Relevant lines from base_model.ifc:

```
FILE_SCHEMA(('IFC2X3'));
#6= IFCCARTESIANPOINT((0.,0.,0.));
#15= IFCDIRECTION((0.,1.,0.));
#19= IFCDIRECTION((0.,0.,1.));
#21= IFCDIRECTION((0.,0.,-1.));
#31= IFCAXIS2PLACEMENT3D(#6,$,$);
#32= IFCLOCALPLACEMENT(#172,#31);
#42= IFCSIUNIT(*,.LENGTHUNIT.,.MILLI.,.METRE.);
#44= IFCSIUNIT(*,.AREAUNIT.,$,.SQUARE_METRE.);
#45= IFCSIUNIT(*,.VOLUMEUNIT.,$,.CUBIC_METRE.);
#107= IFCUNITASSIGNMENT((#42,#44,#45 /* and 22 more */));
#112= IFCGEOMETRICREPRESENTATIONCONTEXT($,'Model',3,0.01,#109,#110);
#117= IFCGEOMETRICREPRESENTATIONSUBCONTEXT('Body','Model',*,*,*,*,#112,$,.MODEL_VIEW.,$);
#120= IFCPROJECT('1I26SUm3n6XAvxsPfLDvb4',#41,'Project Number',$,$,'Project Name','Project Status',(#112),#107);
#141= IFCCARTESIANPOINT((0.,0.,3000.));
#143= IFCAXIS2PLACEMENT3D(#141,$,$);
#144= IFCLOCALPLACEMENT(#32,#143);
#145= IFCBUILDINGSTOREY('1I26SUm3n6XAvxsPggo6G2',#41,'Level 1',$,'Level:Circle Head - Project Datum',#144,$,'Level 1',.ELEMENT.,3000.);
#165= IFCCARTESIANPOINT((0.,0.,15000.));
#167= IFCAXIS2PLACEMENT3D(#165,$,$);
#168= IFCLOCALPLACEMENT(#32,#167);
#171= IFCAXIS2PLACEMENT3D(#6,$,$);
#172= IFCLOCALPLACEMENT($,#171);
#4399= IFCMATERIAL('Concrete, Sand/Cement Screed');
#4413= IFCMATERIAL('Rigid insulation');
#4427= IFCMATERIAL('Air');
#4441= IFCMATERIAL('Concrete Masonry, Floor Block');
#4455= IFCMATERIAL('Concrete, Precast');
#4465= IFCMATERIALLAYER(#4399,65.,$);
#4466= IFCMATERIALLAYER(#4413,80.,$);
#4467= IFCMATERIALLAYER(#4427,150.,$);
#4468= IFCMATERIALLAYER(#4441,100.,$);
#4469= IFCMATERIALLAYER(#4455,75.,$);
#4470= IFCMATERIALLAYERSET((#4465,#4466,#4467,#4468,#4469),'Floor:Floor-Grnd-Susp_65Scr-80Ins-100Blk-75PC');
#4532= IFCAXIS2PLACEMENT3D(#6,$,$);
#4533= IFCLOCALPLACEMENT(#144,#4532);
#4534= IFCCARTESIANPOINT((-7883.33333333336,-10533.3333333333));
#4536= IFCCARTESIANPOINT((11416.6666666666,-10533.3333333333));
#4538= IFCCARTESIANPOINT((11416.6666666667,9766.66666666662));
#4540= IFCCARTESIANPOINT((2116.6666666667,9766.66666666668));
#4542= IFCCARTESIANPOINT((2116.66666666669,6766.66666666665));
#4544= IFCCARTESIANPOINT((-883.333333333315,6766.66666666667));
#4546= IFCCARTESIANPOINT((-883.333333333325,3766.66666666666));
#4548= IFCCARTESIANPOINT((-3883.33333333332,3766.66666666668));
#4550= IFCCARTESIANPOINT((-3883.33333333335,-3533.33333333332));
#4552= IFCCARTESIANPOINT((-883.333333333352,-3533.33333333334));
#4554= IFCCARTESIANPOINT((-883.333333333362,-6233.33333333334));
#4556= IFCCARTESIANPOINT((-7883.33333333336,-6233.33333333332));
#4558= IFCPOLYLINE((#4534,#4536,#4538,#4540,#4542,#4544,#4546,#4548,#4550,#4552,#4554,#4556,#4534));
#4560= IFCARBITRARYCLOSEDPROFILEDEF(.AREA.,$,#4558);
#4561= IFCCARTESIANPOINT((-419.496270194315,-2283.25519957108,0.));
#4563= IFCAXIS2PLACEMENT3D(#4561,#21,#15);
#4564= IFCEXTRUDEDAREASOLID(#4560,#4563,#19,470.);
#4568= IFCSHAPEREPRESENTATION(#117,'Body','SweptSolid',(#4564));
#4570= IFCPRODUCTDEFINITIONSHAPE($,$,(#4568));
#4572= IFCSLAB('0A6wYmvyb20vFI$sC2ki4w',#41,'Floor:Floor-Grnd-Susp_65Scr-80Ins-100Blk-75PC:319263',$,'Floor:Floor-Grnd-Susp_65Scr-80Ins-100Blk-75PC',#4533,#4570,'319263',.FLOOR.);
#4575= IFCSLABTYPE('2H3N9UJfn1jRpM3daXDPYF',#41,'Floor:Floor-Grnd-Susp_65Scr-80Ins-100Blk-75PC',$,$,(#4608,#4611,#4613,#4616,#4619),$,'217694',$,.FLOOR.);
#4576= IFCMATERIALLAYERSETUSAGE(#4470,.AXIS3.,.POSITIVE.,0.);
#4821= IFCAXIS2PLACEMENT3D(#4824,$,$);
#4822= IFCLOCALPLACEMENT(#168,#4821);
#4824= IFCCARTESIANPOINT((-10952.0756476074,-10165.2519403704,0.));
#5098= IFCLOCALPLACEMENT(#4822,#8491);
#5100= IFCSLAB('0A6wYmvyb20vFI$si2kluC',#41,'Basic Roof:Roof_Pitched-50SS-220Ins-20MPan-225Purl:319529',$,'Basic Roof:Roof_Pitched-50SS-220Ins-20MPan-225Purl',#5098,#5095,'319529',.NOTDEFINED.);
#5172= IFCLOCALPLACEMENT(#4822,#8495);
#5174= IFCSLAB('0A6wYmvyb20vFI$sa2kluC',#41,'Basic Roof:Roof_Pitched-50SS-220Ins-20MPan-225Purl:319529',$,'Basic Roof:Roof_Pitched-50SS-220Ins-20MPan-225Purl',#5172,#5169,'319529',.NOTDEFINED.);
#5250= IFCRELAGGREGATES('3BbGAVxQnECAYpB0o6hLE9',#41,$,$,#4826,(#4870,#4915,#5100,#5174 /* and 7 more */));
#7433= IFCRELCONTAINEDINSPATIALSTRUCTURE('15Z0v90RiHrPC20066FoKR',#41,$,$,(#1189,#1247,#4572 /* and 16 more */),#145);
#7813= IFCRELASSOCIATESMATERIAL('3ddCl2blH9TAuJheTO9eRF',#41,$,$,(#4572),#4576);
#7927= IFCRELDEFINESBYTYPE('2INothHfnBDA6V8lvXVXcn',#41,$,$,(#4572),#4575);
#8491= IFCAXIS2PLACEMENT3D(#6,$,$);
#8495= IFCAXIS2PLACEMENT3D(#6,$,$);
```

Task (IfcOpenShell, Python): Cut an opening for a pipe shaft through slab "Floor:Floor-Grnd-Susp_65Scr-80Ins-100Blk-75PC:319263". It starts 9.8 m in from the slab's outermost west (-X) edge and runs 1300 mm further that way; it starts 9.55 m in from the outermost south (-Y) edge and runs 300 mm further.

```python
import numpy as np
import ifcopenshell
import ifcopenshell.api.feature
import ifcopenshell.api.geometry
import ifcopenshell.api.root
import ifcopenshell.geom
import ifcopenshell.util.placement
import ifcopenshell.util.representation
import ifcopenshell.util.shape
import ifcopenshell.util.unit

model = ifcopenshell.open("base_model.ifc")
unit_scale = ifcopenshell.util.unit.calculate_unit_scale(model)
settings = ifcopenshell.geom.settings()


def volume(element):
    """Net volume in cubic metres, openings subtracted."""
    shape = ifcopenshell.geom.create_shape(settings, element)
    return ifcopenshell.util.shape.get_volume(shape.geometry)


slab = model.by_guid("0A6wYmvyb20vFI$sC2ki4w")
before = volume(slab)

# Extent in the slab's own axes, in metres. The edges named are its -X and -Y sides.
slab_shape = ifcopenshell.geom.create_shape(settings, slab)
vertices = ifcopenshell.util.shape.get_vertices(slab_shape.geometry)
x_min, y_min, bottom = vertices.min(axis=0)
top = vertices[:, 2].max()

opening = ifcopenshell.api.root.create_entity(model, ifc_class="IfcOpeningElement", name="Pipe shaft opening")
context = ifcopenshell.util.representation.get_context(model, "Model", "Body", "MODEL_VIEW")
width, depth = 1.3, 0.3
outline = [(0.0, 0.0), (width, 0.0), (width, depth), (0.0, depth), (0.0, 0.0)]
# Overshoot both faces by 50 mm so the cut is clean.
shape = ifcopenshell.api.geometry.add_slab_representation(
    model, context=context, depth=top - bottom + 0.1, polyline=outline
)
ifcopenshell.api.geometry.assign_representation(model, product=opening, representation=shape)

matrix = ifcopenshell.util.placement.get_local_placement(slab.ObjectPlacement)
matrix[:, 3] = matrix @ np.append(np.array([x_min + 9.8, y_min + 9.55, bottom - 0.05]) / unit_scale, 1.0)
ifcopenshell.api.geometry.edit_object_placement(model, product=opening, matrix=matrix, is_si=False)
ifcopenshell.api.feature.add_feature(model, feature=opening, element=slab)

after = volume(slab)

print(f"slab volume {before:.3f} -> {after:.3f} m3")

model.write("base_model-out.ifc")
```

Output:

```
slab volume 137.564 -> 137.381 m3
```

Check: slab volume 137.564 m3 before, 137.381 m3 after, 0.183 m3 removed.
